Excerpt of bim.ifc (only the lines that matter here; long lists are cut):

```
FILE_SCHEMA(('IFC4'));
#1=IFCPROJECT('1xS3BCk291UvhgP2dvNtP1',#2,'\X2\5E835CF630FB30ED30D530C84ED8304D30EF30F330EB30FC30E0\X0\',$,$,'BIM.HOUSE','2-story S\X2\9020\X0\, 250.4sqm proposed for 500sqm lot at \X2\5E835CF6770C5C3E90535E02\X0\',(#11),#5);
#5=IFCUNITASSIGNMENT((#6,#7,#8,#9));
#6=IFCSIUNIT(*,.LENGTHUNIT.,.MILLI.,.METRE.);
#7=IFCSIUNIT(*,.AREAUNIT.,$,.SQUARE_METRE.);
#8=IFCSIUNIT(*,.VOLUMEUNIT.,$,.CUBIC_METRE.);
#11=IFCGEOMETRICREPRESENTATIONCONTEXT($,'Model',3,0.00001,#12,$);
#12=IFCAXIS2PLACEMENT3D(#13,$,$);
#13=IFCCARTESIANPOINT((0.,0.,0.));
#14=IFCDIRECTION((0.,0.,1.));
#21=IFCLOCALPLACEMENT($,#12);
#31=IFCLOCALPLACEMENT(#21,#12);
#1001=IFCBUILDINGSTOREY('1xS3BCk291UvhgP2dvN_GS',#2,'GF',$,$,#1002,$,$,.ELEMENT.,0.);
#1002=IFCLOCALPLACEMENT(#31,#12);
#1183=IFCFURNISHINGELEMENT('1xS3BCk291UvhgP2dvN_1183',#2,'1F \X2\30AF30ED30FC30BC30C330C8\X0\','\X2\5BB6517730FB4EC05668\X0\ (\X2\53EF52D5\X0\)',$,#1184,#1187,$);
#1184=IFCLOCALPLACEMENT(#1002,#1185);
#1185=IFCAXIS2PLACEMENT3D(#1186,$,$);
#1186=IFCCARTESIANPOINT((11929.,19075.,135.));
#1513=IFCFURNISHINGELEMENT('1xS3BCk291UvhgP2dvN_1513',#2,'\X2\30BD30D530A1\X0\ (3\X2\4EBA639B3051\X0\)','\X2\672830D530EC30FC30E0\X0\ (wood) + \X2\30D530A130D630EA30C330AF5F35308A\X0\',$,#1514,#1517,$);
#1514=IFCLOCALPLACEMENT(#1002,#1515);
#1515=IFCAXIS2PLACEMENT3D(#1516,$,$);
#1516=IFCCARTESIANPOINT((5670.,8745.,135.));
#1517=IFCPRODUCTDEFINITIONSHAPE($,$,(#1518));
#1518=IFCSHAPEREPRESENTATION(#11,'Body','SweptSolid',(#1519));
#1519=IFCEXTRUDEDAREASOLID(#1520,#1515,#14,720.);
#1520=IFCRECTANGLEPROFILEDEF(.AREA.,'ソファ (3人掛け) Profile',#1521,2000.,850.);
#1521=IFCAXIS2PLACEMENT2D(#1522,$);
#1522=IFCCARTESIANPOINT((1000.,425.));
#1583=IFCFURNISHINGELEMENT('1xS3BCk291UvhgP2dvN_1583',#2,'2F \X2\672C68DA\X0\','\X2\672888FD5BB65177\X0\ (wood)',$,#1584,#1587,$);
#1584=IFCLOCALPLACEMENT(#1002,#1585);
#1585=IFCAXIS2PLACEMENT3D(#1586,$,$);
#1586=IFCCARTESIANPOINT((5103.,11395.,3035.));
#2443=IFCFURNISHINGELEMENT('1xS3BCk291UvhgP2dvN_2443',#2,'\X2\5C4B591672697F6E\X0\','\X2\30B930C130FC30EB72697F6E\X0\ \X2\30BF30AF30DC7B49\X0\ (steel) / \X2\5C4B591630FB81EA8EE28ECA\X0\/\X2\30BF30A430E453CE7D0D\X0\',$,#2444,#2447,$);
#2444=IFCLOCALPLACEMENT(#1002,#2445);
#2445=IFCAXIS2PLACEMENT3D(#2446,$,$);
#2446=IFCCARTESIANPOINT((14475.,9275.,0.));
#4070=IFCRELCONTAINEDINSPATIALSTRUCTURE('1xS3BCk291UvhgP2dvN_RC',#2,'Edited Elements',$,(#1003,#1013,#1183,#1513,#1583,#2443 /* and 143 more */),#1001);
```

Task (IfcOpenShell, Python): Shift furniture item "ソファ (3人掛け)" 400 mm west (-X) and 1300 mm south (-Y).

```python
import ifcopenshell
import ifcopenshell.api.geometry
import ifcopenshell.util.placement
import ifcopenshell.util.unit

model = ifcopenshell.open("bim.ifc")
unit_scale = ifcopenshell.util.unit.calculate_unit_scale(model)

item = model.by_guid("1xS3BCk291UvhgP2dvN_1513")
matrix = ifcopenshell.util.placement.get_local_placement(item.ObjectPlacement)
matrix[0, 3] -= 0.4 / unit_scale
matrix[1, 3] -= 1.3 / unit_scale
ifcopenshell.api.geometry.edit_object_placement(model, product=item, matrix=matrix, is_si=False)

print(ifcopenshell.util.placement.get_local_placement(item.ObjectPlacement).round(3) + 0.0)

model.write("bim_rev.ifc")
```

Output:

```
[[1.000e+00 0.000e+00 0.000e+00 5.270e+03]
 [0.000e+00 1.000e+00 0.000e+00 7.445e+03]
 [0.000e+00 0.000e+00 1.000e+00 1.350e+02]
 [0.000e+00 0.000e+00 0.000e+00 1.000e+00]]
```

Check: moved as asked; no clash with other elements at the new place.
